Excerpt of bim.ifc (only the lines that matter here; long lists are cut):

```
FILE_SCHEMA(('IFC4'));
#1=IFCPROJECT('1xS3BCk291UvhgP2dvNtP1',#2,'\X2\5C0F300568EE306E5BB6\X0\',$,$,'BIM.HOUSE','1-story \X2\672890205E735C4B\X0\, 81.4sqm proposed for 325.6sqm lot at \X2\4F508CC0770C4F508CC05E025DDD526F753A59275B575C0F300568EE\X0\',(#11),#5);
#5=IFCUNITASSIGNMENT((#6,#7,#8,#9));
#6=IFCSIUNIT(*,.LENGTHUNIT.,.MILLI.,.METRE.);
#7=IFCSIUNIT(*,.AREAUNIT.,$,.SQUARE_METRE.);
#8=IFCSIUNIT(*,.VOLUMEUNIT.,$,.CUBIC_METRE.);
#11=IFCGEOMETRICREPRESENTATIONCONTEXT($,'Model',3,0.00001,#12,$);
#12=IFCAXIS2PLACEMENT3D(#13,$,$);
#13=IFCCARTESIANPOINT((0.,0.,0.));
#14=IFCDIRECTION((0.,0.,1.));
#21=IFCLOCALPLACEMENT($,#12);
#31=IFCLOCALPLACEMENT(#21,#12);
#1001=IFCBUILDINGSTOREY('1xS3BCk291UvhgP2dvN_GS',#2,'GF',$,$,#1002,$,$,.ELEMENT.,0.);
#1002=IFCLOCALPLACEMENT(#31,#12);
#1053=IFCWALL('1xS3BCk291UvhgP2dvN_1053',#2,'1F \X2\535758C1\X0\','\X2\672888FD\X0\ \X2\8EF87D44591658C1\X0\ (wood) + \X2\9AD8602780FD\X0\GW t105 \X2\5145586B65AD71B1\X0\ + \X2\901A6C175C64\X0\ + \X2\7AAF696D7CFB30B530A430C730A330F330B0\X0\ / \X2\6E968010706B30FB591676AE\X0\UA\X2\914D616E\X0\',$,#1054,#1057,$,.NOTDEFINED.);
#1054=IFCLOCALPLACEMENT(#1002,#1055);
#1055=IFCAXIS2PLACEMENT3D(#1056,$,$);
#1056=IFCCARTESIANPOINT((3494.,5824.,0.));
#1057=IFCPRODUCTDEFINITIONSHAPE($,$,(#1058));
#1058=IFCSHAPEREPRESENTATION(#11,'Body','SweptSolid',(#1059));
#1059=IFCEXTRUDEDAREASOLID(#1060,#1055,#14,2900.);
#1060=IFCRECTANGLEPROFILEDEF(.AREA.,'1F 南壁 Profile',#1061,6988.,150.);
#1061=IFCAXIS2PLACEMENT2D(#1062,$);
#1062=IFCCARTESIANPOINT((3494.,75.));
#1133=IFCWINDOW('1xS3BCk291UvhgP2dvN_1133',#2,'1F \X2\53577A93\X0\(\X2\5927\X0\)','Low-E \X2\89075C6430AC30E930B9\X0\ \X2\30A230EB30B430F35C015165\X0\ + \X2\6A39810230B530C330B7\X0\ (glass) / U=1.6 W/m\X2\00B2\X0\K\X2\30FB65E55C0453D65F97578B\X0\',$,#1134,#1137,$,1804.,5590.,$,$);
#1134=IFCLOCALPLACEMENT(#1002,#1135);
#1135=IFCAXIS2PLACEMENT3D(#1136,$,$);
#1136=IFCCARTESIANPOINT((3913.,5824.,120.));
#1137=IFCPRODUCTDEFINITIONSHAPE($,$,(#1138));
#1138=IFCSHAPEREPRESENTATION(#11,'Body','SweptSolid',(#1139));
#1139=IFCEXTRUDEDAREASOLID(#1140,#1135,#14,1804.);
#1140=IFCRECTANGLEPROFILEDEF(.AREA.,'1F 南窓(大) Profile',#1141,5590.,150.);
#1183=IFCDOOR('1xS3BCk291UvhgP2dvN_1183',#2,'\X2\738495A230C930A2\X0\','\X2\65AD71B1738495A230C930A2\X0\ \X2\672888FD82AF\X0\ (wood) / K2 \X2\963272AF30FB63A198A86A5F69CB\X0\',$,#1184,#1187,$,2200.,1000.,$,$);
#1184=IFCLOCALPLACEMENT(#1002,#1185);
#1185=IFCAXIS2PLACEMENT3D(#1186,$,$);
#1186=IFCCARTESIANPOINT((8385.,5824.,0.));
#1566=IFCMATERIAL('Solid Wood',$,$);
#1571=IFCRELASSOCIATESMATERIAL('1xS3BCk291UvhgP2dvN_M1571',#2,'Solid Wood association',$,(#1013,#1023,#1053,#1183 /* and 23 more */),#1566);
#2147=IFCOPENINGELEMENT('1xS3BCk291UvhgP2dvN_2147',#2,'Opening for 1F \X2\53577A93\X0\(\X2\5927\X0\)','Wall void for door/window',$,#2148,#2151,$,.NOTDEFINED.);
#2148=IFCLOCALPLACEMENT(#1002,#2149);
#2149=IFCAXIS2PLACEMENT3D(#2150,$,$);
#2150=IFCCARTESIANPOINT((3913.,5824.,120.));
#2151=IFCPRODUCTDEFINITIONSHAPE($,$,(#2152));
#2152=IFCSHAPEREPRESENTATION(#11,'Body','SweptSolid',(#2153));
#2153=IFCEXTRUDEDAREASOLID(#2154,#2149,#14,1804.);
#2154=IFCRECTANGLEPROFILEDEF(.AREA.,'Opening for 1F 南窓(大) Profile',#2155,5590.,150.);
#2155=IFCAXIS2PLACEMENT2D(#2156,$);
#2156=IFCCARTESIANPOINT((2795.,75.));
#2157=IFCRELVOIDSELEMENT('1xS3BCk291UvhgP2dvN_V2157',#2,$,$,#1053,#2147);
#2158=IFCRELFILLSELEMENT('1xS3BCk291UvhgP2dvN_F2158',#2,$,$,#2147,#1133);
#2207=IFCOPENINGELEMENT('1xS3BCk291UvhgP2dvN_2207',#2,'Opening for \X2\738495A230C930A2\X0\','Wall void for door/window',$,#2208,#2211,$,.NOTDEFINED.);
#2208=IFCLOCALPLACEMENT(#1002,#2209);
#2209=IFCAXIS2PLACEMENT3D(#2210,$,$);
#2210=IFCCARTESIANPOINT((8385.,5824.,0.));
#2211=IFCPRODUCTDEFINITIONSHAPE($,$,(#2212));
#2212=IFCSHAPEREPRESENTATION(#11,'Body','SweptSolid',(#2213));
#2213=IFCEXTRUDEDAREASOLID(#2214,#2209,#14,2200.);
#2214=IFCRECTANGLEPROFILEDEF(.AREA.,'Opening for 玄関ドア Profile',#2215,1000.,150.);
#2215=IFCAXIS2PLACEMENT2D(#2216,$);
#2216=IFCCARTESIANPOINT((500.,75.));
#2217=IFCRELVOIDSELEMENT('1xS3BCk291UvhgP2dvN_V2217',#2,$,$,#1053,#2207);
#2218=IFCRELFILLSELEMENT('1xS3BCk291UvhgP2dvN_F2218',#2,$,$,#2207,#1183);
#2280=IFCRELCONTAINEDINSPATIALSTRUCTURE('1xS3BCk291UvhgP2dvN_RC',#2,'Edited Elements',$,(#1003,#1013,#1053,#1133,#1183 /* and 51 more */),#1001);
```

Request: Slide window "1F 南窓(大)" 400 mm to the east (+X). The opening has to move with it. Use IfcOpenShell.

```python
import ifcopenshell
import ifcopenshell.api.geometry
import ifcopenshell.util.placement

model = ifcopenshell.open("bim.ifc")

window = model.by_guid("1xS3BCk291UvhgP2dvN_1133")
opening = window.FillsVoids[0].RelatingOpeningElement
wall = opening.VoidsElements[0].RelatingBuildingElement

wall_matrix = ifcopenshell.util.placement.get_local_placement(wall.ObjectPlacement)
shift = wall_matrix[:3, 0] * 400.0
before = ifcopenshell.util.placement.get_local_placement(window.ObjectPlacement)[:3, 3].copy()

# The window is not placed relative to its opening, so move both.
for product in (opening, window):
    matrix = ifcopenshell.util.placement.get_local_placement(product.ObjectPlacement)
    matrix[:3, 3] += shift
    ifcopenshell.api.geometry.edit_object_placement(model, product=product, matrix=matrix, is_si=False)

after = ifcopenshell.util.placement.get_local_placement(window.ObjectPlacement)[:3, 3]
print("window moved by", (after - before).round(3) + 0.0)

model.write("bim_edited.ifc")
```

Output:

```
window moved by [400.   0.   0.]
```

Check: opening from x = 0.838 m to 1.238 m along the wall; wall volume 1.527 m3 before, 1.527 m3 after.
